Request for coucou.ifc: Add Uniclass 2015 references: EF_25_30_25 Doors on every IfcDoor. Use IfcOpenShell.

First a look at what the model holds.

```python
import ifcopenshell

model = ifcopenshell.open("coucou.ifc")
print(model.schema)
print("classifications:", [c.Name for c in model.by_type("IfcClassification")])
for ifc_class in ("IfcDoor", "IfcRoof", "IfcStair", "IfcWall", "IfcWindow"):
    print(ifc_class, len(model.by_type(ifc_class)))
```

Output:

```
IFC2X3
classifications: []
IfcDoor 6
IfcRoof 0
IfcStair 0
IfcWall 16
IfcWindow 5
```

```python
import ifcopenshell
import ifcopenshell.api.classification

model = ifcopenshell.open("coucou.ifc")

# IFC2X3 requires Source and Edition and has no link from the project to the system.
system = model.create_entity("IfcClassification", Source="NBS", Edition="2015", Name="Uniclass 2015")

codes = {
    "IfcDoor": ("EF_25_30_25", "Doors"),
}
for ifc_class, (code, name) in codes.items():
    products = model.by_type(ifc_class)
    ifcopenshell.api.classification.add_reference(
        model, products=products, classification=system, identification=code, name=name
    )
    print(code, len(products))

model.write("coucou_edited.ifc")
```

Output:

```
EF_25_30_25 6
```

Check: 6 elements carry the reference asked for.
